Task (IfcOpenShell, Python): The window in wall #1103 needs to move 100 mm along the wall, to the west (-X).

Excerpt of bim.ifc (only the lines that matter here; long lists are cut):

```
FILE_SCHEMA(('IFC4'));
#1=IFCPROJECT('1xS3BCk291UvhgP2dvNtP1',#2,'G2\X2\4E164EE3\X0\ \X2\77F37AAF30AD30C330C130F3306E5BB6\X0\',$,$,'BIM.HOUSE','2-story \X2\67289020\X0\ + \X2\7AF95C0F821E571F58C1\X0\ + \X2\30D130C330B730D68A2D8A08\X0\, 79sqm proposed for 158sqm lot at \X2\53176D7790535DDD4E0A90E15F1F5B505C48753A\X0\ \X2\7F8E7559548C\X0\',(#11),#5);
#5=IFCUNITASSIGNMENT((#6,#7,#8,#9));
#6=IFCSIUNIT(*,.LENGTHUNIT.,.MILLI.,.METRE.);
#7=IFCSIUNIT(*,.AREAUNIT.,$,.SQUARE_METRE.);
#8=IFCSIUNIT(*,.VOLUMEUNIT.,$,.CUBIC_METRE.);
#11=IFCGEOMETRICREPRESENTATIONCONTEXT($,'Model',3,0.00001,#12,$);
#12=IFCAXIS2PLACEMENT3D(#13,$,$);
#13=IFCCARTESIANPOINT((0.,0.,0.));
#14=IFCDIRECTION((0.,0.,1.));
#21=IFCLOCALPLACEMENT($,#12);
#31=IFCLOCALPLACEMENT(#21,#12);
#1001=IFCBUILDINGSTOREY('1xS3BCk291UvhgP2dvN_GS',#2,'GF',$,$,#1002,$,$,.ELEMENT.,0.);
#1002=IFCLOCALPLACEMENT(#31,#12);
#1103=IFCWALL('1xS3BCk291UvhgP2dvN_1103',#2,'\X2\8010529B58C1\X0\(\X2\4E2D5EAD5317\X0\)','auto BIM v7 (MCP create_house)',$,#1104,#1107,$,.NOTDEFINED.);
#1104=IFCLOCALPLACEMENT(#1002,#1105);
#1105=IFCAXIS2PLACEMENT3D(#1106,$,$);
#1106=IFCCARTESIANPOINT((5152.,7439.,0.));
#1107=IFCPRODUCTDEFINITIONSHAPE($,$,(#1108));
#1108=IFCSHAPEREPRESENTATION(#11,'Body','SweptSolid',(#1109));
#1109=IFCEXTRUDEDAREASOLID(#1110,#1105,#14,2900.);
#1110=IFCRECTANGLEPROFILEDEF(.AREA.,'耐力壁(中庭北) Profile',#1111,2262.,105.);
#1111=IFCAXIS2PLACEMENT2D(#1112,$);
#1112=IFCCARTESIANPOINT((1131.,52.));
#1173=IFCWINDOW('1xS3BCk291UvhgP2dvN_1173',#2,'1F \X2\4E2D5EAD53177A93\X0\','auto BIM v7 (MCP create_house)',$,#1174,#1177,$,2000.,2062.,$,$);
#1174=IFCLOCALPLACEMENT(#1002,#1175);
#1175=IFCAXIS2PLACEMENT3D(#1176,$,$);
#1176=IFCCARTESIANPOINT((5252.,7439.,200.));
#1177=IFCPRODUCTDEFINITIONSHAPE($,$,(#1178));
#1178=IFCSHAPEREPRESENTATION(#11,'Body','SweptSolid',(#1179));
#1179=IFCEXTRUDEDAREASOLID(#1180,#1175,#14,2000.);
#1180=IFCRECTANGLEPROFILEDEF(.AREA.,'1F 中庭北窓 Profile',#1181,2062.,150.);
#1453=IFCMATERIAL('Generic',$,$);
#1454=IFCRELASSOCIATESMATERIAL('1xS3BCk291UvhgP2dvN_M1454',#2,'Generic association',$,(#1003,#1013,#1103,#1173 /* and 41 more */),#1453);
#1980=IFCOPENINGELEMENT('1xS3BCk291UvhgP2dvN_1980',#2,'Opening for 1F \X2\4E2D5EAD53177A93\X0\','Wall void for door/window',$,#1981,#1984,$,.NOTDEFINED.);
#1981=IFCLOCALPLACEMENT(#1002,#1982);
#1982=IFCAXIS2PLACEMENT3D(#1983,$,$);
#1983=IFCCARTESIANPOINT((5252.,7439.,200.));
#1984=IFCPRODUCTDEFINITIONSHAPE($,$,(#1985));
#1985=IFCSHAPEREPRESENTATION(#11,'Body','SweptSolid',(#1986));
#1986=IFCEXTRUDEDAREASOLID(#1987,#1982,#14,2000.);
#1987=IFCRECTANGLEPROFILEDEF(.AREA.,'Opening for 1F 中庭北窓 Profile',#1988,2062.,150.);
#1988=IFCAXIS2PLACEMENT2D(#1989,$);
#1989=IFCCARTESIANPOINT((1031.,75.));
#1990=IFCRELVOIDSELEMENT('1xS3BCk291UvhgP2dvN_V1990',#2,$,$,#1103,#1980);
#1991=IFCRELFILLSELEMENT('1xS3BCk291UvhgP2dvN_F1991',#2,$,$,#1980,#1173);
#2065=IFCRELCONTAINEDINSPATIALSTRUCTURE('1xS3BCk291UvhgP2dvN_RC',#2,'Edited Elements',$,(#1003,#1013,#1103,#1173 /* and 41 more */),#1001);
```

```python
import ifcopenshell
import ifcopenshell.api.geometry
import ifcopenshell.util.placement

model = ifcopenshell.open("bim.ifc")

window = model.by_guid("1xS3BCk291UvhgP2dvN_1173")
opening = window.FillsVoids[0].RelatingOpeningElement
wall = opening.VoidsElements[0].RelatingBuildingElement

wall_matrix = ifcopenshell.util.placement.get_local_placement(wall.ObjectPlacement)
shift = wall_matrix[:3, 0] * -100.0
before = ifcopenshell.util.placement.get_local_placement(window.ObjectPlacement)[:3, 3].copy()

# The window is not placed relative to its opening, so move both.
for product in (opening, window):
    matrix = ifcopenshell.util.placement.get_local_placement(product.ObjectPlacement)
    matrix[:3, 3] += shift
    ifcopenshell.api.geometry.edit_object_placement(model, product=product, matrix=matrix, is_si=False)

after = ifcopenshell.util.placement.get_local_placement(window.ObjectPlacement)[:3, 3]
print("window moved by", (after - before).round(3) + 0.0)

model.write("bim_rev.ifc")
```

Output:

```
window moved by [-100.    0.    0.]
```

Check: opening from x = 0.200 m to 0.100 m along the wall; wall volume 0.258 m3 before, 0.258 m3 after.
